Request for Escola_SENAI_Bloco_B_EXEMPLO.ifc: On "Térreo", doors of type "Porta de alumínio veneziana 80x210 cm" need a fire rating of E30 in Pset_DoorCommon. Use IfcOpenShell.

First a look at what the model holds.

```python
import ifcopenshell
import ifcopenshell.util.element

model = ifcopenshell.open("Escola_SENAI_Bloco_B_EXEMPLO.ifc")
print(model.schema)
storey = next(s for s in model.by_type("IfcBuildingStorey") if s.Name == "Térreo")
doors = [e for e in ifcopenshell.util.element.get_decomposition(storey) if e.is_a("IfcDoor")]
seen = {}
for e in doors:
    element_type = ifcopenshell.util.element.get_type(e)
    key = (element_type.Name if element_type != e and element_type else None, ifcopenshell.util.element.get_pset(e, "Pset_DoorCommon", "FireRating"))
    seen[key] = seen.get(key, 0) + 1
for (name, value), count in sorted(seen.items(), key=str):
    print(count, "x", name, "|", value)
```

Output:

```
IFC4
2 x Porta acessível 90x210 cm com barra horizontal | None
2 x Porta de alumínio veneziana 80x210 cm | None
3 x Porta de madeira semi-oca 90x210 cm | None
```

```python
import ifcopenshell
import ifcopenshell.api.pset
import ifcopenshell.util.element

model = ifcopenshell.open("Escola_SENAI_Bloco_B_EXEMPLO.ifc")

storey = next(s for s in model.by_type("IfcBuildingStorey") if s.Name == "Térreo")
doors = [e for e in ifcopenshell.util.element.get_decomposition(storey) if e.is_a("IfcDoor")]

count = 0
for e in doors:
    element_type = ifcopenshell.util.element.get_type(e)
    if element_type in (None, e) or element_type.Name != "Porta de alumínio veneziana 80x210 cm":
        continue
    # add_pset returns the element's existing set when there is one.
    pset = ifcopenshell.api.pset.add_pset(model, product=e, name="Pset_DoorCommon")
    ifcopenshell.api.pset.edit_pset(model, pset=pset, properties={"FireRating": "E30"})
    count += 1

print(count, "doors updated")

model.write("Escola_SENAI_Bloco_B_EXEMPLO_rev.ifc")
```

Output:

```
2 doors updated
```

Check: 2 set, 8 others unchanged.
